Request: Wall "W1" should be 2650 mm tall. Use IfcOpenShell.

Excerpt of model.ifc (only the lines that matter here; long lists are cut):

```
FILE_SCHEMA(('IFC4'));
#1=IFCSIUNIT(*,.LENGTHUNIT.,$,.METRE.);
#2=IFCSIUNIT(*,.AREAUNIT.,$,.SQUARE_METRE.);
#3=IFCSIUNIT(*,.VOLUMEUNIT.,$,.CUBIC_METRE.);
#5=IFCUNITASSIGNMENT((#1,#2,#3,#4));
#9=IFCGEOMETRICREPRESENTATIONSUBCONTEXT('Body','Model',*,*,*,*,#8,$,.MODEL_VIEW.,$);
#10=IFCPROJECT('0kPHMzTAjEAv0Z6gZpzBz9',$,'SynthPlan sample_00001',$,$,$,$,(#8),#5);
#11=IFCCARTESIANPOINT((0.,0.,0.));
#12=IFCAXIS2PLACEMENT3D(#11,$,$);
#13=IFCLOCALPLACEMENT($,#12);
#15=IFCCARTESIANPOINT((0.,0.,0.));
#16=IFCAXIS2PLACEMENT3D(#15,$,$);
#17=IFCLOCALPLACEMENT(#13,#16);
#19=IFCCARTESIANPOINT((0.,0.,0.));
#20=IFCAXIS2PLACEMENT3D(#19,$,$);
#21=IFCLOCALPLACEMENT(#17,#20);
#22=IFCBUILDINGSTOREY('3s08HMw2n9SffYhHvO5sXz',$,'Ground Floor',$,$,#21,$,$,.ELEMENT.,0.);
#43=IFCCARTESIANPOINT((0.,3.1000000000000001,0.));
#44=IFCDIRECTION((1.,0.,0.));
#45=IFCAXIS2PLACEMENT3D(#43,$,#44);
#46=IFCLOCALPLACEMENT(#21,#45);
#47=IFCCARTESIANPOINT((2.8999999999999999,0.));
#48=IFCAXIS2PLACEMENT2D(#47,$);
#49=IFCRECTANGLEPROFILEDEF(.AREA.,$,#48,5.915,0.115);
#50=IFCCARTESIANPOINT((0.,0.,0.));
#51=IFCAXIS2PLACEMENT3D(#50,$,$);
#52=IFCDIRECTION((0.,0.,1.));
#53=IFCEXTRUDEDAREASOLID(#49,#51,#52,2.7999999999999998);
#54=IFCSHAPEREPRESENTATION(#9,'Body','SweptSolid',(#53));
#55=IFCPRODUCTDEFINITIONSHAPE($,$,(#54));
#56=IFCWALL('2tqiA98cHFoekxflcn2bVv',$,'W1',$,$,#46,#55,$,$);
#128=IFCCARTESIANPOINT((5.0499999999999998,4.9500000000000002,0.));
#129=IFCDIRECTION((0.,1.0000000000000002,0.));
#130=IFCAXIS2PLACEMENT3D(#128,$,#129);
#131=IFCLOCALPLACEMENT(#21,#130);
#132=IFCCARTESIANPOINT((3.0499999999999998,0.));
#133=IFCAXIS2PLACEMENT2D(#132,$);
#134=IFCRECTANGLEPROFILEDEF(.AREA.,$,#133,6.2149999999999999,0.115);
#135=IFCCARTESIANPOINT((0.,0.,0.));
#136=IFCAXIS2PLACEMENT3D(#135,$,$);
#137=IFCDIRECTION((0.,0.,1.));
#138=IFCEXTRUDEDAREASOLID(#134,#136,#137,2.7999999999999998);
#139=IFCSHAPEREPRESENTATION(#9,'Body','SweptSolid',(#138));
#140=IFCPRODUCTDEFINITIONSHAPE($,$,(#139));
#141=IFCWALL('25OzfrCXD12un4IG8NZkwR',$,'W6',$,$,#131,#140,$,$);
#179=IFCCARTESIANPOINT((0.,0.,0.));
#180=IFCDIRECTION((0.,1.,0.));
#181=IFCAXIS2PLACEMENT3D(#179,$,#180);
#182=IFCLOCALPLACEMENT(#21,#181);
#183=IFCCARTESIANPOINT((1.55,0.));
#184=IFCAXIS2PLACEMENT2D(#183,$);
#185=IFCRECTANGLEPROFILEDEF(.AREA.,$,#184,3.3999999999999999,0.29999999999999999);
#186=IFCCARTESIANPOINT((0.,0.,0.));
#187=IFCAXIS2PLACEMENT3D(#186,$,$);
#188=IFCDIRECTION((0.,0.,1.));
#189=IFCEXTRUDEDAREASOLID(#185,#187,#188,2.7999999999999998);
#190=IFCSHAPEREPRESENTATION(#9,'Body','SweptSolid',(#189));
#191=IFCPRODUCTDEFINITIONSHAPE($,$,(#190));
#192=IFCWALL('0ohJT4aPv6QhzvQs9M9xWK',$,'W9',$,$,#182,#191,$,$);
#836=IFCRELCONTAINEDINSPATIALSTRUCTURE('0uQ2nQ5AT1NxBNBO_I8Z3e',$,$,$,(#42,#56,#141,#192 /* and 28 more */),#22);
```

```python
import ifcopenshell
import ifcopenshell.geom
import ifcopenshell.util.representation
import ifcopenshell.util.shape
import ifcopenshell.util.unit

model = ifcopenshell.open("model.ifc")
unit_scale = ifcopenshell.util.unit.calculate_unit_scale(model)
settings = ifcopenshell.geom.settings()


def volume(element):
    """Net volume in cubic metres, openings subtracted."""
    shape = ifcopenshell.geom.create_shape(settings, element)
    return ifcopenshell.util.shape.get_volume(shape.geometry)


wall = model.by_guid("2tqiA98cHFoekxflcn2bVv")
before = volume(wall)

body = ifcopenshell.util.representation.get_representation(wall, "Model", "Body")
solid = body.Items[0]
old_height = solid.Depth
solid.Depth = 2.65 / unit_scale
after = volume(wall)

print(f"height {old_height:g} -> {solid.Depth:g}, volume {before:.3f} -> {after:.3f} m3")

model.write("model_rev.ifc")
```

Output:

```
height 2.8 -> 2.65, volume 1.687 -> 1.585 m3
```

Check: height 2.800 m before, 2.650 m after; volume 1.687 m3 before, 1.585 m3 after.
